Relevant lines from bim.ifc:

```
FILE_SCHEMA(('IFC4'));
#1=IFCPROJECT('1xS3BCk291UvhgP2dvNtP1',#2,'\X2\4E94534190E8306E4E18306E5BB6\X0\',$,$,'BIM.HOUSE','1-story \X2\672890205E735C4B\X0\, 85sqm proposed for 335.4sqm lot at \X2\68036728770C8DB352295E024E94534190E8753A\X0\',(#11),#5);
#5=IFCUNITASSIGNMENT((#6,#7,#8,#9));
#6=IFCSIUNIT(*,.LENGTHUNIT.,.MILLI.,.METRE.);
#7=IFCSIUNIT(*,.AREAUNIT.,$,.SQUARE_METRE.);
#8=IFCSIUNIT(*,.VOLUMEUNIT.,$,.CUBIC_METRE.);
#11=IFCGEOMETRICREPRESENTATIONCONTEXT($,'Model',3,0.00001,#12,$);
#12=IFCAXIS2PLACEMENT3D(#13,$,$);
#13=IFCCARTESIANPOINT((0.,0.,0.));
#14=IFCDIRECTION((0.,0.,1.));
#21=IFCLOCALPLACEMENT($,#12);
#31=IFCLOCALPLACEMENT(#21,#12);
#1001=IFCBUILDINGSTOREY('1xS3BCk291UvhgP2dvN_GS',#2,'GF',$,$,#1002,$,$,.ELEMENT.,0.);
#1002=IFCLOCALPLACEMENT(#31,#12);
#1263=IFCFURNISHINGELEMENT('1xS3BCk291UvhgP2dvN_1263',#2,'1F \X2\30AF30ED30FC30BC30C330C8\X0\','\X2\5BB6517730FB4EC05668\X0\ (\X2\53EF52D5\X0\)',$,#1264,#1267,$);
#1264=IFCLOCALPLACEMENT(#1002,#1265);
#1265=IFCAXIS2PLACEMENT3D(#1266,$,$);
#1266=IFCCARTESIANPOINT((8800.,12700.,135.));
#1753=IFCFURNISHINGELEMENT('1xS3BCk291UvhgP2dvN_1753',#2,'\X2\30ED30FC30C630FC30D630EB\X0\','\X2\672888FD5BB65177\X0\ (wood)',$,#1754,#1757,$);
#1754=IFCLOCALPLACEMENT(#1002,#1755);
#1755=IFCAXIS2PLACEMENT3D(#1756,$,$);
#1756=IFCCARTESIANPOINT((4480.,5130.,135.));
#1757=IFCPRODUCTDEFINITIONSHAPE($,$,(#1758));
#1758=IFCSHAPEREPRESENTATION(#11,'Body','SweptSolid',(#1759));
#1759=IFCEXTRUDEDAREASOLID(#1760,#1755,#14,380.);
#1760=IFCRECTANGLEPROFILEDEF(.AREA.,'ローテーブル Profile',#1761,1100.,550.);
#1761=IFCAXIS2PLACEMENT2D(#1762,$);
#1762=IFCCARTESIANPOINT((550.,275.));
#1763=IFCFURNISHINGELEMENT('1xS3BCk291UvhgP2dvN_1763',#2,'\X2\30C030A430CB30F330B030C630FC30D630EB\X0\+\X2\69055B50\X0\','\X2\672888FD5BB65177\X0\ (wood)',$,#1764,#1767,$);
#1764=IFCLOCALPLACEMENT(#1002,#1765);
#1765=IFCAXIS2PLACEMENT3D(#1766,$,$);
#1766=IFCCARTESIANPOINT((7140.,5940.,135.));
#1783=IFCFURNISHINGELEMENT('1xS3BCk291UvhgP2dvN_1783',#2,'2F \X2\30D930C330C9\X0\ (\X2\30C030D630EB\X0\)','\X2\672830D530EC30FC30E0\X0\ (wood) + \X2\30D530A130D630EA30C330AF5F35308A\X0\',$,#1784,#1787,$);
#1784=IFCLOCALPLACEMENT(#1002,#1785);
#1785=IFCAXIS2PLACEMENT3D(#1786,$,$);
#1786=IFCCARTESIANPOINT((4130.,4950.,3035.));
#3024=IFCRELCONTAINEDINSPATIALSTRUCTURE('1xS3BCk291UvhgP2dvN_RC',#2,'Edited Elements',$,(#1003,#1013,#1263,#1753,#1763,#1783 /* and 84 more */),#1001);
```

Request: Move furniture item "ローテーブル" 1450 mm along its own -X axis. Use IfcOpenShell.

```python
import ifcopenshell
import ifcopenshell.api.geometry
import ifcopenshell.util.placement

model = ifcopenshell.open("bim.ifc")

item = model.by_guid("1xS3BCk291UvhgP2dvN_1753")
matrix = ifcopenshell.util.placement.get_local_placement(item.ObjectPlacement)
matrix[:3, 3] -= matrix[:3, 0] * 1450.0
ifcopenshell.api.geometry.edit_object_placement(model, product=item, matrix=matrix, is_si=False)

print(ifcopenshell.util.placement.get_local_placement(item.ObjectPlacement).round(3) + 0.0)

model.write("bim_v2.ifc")
```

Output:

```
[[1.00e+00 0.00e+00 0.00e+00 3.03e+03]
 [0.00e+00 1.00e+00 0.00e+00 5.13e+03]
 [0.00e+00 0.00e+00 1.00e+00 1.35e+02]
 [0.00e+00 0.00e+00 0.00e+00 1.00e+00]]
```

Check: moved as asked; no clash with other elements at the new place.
